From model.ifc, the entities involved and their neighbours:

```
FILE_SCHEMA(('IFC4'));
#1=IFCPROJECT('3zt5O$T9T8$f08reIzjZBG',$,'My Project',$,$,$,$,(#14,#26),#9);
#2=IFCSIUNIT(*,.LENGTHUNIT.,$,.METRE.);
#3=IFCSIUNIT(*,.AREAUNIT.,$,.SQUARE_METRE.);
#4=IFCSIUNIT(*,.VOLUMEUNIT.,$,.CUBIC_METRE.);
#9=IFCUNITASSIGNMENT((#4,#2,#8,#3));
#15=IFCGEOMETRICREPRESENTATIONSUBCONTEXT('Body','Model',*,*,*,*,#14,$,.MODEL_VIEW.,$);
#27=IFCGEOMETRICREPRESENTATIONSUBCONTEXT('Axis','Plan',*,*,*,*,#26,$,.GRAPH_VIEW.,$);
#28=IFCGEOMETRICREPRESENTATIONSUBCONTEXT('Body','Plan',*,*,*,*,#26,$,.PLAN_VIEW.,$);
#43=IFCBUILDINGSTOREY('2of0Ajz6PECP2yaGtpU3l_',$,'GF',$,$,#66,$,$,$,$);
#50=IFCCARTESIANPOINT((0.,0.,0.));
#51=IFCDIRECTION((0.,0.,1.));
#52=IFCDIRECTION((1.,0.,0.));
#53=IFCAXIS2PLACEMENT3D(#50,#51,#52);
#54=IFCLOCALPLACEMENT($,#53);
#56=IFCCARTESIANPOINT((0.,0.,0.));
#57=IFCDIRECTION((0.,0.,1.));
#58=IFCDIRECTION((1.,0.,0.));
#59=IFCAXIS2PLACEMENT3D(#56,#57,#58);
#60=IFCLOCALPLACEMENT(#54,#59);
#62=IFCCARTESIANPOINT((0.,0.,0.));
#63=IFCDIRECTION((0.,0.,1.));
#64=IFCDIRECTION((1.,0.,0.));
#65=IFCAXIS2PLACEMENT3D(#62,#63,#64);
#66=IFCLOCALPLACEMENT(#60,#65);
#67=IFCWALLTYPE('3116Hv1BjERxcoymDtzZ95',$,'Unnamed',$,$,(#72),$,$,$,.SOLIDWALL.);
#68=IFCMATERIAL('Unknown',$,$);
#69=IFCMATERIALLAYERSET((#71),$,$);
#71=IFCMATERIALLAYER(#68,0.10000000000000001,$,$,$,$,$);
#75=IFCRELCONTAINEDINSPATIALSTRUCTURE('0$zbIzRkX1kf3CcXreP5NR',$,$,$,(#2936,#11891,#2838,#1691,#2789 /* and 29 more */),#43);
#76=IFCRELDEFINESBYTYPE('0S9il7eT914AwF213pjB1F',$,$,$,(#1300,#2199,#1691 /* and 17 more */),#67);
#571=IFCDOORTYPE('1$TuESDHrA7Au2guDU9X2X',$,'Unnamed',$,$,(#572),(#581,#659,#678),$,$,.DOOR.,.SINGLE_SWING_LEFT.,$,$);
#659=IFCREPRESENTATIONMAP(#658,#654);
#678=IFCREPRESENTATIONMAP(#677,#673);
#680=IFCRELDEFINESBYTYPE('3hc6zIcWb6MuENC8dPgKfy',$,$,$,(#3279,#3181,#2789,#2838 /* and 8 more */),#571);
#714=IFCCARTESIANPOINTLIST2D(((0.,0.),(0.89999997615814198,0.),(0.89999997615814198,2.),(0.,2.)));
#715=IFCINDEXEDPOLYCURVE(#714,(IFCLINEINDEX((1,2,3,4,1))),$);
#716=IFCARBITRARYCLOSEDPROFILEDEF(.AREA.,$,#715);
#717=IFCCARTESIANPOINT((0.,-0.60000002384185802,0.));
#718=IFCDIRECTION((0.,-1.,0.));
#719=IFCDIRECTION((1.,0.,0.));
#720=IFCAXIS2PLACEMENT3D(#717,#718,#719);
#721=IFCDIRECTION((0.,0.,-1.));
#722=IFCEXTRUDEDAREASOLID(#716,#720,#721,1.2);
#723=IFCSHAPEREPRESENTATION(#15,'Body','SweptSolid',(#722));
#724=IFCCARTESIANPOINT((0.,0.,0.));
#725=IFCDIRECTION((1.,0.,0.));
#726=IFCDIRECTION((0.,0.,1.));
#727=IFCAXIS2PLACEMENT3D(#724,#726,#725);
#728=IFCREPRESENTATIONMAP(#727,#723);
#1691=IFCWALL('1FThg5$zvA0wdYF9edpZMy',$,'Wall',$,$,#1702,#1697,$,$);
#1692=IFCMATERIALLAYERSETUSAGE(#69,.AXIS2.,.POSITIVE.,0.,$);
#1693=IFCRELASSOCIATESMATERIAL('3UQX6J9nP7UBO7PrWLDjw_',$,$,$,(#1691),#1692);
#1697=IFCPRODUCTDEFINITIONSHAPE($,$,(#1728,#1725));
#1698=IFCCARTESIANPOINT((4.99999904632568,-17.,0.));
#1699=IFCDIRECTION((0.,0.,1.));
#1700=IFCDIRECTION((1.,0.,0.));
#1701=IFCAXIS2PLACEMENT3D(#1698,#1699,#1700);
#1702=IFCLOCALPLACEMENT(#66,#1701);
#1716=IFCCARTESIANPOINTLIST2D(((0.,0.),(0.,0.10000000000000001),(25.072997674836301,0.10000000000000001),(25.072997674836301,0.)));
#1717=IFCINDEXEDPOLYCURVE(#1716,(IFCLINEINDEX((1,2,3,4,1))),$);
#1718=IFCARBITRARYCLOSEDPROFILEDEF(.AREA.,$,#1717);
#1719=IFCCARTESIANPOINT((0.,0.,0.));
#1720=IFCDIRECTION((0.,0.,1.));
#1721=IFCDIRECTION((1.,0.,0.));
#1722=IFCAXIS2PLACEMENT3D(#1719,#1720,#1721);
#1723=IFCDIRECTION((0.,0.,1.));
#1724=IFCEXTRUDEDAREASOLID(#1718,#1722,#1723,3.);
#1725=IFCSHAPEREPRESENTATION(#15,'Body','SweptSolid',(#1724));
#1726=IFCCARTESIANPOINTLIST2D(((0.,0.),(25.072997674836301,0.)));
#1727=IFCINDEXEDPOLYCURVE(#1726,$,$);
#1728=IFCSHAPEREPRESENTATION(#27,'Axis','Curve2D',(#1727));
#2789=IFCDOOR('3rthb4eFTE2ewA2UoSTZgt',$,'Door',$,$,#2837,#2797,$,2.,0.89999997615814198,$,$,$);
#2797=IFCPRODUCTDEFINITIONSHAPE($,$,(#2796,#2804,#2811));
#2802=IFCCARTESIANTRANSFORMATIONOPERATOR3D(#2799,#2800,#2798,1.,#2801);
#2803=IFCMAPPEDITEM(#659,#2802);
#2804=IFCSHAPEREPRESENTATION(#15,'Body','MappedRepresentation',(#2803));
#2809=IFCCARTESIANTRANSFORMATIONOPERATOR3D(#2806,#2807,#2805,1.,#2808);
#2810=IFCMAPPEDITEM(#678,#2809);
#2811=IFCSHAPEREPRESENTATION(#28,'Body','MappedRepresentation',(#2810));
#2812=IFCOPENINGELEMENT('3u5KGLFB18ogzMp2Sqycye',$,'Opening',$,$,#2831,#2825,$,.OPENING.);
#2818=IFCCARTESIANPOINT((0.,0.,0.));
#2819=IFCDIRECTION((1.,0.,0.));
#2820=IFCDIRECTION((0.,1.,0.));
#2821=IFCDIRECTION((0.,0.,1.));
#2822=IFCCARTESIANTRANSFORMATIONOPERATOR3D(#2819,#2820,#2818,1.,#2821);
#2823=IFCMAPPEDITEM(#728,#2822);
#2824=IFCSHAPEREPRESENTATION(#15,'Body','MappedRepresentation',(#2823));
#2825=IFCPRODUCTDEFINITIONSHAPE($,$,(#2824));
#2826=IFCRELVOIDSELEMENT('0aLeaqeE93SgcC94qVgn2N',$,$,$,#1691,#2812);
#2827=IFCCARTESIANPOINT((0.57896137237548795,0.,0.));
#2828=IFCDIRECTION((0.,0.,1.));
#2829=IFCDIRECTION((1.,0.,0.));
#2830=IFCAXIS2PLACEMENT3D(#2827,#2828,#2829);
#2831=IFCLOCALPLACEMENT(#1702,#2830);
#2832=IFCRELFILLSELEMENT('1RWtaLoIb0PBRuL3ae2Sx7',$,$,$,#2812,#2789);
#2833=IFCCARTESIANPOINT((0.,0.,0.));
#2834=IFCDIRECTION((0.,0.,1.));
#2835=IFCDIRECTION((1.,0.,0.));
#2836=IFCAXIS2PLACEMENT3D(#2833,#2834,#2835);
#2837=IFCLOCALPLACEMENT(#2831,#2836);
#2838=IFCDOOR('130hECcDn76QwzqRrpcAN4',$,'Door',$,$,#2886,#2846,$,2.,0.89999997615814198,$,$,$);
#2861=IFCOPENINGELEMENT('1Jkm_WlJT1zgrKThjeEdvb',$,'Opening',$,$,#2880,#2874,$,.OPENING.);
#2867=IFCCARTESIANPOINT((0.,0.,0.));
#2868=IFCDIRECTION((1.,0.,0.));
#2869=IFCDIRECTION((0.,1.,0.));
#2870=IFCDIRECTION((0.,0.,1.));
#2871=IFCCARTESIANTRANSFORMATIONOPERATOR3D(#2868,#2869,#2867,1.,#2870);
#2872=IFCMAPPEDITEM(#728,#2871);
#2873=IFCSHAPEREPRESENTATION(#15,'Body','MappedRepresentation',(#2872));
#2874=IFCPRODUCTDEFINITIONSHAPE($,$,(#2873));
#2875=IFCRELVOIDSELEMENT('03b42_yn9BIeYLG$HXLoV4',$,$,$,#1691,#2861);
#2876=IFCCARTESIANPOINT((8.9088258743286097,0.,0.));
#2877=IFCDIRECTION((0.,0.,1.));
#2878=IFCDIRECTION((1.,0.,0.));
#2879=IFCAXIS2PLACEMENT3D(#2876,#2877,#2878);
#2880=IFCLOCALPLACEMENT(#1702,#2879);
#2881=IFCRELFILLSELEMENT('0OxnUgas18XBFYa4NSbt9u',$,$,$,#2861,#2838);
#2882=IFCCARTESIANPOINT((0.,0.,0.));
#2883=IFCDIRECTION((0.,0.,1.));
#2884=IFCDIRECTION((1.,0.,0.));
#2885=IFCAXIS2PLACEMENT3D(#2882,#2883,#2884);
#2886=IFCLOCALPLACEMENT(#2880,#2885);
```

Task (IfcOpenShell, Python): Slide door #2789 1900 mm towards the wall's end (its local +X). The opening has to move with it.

```python
import ifcopenshell
import ifcopenshell.api.geometry
import ifcopenshell.util.placement
import ifcopenshell.util.unit

model = ifcopenshell.open("model.ifc")
unit_scale = ifcopenshell.util.unit.calculate_unit_scale(model)

door = model.by_guid("3rthb4eFTE2ewA2UoSTZgt")
opening = door.FillsVoids[0].RelatingOpeningElement
wall = opening.VoidsElements[0].RelatingBuildingElement

wall_matrix = ifcopenshell.util.placement.get_local_placement(wall.ObjectPlacement)
shift = wall_matrix[:3, 0] * 1.9 / unit_scale
before = ifcopenshell.util.placement.get_local_placement(door.ObjectPlacement)[:3, 3].copy()

# The door is placed relative to its opening, so it follows when the opening moves.
matrix = ifcopenshell.util.placement.get_local_placement(opening.ObjectPlacement)
matrix[:3, 3] += shift
ifcopenshell.api.geometry.edit_object_placement(
    model, product=opening, matrix=matrix, is_si=False, should_transform_children=True
)

after = ifcopenshell.util.placement.get_local_placement(door.ObjectPlacement)[:3, 3]
print("door moved by", (after - before).round(3) + 0.0)

model.write("model_rev.ifc")
```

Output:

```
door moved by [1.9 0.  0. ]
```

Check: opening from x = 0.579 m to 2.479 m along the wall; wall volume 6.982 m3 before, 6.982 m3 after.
